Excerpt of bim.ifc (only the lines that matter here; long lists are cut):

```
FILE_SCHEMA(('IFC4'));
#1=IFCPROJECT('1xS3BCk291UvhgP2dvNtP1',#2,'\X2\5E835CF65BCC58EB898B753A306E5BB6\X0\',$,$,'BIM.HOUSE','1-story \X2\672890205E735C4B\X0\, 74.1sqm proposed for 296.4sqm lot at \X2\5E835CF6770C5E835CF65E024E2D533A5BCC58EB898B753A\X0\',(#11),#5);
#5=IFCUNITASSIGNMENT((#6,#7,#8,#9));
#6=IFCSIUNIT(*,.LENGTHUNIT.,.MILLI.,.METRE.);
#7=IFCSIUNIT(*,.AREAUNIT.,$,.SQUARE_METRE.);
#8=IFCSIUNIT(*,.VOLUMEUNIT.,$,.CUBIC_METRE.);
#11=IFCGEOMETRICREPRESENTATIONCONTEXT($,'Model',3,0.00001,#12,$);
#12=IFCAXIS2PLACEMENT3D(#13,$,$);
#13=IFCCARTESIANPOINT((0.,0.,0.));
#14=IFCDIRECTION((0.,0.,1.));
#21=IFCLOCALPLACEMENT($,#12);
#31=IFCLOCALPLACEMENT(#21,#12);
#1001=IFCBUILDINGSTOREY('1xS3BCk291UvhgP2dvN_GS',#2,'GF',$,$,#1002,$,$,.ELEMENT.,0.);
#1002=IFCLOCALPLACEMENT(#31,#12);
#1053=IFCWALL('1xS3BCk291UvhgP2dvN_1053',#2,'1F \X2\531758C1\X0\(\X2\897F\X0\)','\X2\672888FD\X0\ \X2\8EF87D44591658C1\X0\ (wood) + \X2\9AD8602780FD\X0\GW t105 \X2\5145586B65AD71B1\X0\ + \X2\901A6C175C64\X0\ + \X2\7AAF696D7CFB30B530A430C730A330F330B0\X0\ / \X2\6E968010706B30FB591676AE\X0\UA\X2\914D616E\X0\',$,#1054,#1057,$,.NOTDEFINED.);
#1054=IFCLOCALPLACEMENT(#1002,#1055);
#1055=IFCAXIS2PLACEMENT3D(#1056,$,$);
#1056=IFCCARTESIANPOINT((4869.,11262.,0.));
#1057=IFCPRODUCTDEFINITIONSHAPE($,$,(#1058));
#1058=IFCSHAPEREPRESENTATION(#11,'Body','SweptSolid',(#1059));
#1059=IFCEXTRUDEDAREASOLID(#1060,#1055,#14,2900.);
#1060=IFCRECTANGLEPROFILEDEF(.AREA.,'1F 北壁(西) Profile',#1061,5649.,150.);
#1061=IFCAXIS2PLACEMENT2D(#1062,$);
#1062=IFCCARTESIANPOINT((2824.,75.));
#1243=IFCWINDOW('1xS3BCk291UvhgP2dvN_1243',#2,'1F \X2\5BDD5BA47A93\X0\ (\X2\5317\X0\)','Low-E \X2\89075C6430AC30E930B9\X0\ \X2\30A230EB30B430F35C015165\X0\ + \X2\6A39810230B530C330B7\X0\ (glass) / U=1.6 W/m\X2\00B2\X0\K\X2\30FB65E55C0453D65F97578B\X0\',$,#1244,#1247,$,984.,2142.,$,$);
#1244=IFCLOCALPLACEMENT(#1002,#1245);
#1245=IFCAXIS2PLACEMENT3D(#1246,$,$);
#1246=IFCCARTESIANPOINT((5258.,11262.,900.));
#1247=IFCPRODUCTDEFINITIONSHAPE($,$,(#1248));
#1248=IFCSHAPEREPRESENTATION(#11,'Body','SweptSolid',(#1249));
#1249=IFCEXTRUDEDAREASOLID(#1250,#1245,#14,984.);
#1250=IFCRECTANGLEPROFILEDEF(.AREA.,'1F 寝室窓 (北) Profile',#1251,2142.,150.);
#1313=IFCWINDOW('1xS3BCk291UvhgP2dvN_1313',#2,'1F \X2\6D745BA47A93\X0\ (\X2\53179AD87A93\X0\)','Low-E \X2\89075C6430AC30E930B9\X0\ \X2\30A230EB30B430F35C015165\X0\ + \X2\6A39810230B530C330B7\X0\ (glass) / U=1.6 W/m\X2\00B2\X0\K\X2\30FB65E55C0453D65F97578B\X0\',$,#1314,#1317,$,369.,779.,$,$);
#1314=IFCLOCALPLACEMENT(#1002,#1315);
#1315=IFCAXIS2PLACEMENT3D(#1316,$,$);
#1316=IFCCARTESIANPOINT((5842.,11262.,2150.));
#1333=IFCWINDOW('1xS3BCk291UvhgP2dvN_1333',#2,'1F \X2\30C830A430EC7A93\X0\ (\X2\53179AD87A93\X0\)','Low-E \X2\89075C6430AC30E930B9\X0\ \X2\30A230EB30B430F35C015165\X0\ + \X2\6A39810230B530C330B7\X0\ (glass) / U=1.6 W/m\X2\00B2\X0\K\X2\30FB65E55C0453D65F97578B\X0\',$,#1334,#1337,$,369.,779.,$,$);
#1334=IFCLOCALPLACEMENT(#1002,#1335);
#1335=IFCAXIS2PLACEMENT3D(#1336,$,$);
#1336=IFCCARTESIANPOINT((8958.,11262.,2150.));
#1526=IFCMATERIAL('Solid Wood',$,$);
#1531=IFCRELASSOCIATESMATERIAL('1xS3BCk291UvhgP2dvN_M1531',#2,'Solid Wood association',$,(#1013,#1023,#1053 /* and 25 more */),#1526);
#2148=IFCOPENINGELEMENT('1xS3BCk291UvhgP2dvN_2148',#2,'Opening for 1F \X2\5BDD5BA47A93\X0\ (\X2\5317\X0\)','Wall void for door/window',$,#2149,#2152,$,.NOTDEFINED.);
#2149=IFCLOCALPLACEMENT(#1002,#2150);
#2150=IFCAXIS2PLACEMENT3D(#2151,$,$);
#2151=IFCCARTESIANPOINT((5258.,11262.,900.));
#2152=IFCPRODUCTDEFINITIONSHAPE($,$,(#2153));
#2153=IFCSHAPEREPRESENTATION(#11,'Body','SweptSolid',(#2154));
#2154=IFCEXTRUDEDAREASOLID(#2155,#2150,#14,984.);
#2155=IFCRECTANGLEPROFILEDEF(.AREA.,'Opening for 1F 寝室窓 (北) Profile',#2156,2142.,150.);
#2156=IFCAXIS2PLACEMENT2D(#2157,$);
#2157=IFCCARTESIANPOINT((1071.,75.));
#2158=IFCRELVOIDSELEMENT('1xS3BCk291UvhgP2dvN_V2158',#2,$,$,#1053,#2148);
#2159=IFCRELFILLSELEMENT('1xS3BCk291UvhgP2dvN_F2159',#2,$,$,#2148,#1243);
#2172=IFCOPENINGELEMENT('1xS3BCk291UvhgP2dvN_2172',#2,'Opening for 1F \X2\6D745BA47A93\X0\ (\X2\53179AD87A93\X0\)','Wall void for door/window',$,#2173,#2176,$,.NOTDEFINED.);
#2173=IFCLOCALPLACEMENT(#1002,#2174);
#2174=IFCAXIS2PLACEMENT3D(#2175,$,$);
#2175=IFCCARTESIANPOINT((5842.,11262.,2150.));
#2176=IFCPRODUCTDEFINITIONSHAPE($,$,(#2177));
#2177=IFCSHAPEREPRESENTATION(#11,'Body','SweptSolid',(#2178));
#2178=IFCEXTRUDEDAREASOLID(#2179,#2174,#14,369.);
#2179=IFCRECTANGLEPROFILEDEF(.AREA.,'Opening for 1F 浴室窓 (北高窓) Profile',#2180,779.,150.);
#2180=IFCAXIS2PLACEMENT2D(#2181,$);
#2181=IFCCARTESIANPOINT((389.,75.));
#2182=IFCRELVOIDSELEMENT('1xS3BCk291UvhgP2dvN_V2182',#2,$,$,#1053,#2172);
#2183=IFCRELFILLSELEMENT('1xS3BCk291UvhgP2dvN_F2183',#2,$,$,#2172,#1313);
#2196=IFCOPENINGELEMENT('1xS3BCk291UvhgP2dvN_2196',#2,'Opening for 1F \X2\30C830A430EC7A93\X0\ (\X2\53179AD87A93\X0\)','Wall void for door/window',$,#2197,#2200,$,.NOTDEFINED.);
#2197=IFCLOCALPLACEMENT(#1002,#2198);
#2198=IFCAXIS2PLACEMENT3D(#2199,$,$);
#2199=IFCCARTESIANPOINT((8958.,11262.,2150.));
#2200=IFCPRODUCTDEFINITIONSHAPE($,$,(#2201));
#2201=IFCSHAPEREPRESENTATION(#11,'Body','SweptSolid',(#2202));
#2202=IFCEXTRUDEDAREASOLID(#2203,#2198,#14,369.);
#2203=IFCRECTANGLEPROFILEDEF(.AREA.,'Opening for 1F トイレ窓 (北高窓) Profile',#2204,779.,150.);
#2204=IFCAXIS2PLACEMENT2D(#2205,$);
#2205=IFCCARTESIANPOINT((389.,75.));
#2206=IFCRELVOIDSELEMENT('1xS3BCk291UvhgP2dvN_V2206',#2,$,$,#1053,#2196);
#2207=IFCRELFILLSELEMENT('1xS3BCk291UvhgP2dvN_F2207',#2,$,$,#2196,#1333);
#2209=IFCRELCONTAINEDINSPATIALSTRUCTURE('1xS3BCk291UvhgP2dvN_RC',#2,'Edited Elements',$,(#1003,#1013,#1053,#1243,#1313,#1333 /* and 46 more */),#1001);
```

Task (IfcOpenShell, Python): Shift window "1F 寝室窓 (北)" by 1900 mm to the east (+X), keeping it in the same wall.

```python
import ifcopenshell
import ifcopenshell.api.geometry
import ifcopenshell.util.placement
import ifcopenshell.util.unit

model = ifcopenshell.open("bim.ifc")
unit_scale = ifcopenshell.util.unit.calculate_unit_scale(model)

window = model.by_guid("1xS3BCk291UvhgP2dvN_1243")
opening = window.FillsVoids[0].RelatingOpeningElement
wall = opening.VoidsElements[0].RelatingBuildingElement

wall_matrix = ifcopenshell.util.placement.get_local_placement(wall.ObjectPlacement)
shift = wall_matrix[:3, 0] * 1.9 / unit_scale
before = ifcopenshell.util.placement.get_local_placement(window.ObjectPlacement)[:3, 3].copy()

# The window is not placed relative to its opening, so move both.
for product in (opening, window):
    matrix = ifcopenshell.util.placement.get_local_placement(product.ObjectPlacement)
    matrix[:3, 3] += shift
    ifcopenshell.api.geometry.edit_object_placement(model, product=product, matrix=matrix, is_si=False)

after = ifcopenshell.util.placement.get_local_placement(window.ObjectPlacement)[:3, 3]
print("window moved by", (after - before).round(3) + 0.0)

model.write("bim_edited.ifc")
```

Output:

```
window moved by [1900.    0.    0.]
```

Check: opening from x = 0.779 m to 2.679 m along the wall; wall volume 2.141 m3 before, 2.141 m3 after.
